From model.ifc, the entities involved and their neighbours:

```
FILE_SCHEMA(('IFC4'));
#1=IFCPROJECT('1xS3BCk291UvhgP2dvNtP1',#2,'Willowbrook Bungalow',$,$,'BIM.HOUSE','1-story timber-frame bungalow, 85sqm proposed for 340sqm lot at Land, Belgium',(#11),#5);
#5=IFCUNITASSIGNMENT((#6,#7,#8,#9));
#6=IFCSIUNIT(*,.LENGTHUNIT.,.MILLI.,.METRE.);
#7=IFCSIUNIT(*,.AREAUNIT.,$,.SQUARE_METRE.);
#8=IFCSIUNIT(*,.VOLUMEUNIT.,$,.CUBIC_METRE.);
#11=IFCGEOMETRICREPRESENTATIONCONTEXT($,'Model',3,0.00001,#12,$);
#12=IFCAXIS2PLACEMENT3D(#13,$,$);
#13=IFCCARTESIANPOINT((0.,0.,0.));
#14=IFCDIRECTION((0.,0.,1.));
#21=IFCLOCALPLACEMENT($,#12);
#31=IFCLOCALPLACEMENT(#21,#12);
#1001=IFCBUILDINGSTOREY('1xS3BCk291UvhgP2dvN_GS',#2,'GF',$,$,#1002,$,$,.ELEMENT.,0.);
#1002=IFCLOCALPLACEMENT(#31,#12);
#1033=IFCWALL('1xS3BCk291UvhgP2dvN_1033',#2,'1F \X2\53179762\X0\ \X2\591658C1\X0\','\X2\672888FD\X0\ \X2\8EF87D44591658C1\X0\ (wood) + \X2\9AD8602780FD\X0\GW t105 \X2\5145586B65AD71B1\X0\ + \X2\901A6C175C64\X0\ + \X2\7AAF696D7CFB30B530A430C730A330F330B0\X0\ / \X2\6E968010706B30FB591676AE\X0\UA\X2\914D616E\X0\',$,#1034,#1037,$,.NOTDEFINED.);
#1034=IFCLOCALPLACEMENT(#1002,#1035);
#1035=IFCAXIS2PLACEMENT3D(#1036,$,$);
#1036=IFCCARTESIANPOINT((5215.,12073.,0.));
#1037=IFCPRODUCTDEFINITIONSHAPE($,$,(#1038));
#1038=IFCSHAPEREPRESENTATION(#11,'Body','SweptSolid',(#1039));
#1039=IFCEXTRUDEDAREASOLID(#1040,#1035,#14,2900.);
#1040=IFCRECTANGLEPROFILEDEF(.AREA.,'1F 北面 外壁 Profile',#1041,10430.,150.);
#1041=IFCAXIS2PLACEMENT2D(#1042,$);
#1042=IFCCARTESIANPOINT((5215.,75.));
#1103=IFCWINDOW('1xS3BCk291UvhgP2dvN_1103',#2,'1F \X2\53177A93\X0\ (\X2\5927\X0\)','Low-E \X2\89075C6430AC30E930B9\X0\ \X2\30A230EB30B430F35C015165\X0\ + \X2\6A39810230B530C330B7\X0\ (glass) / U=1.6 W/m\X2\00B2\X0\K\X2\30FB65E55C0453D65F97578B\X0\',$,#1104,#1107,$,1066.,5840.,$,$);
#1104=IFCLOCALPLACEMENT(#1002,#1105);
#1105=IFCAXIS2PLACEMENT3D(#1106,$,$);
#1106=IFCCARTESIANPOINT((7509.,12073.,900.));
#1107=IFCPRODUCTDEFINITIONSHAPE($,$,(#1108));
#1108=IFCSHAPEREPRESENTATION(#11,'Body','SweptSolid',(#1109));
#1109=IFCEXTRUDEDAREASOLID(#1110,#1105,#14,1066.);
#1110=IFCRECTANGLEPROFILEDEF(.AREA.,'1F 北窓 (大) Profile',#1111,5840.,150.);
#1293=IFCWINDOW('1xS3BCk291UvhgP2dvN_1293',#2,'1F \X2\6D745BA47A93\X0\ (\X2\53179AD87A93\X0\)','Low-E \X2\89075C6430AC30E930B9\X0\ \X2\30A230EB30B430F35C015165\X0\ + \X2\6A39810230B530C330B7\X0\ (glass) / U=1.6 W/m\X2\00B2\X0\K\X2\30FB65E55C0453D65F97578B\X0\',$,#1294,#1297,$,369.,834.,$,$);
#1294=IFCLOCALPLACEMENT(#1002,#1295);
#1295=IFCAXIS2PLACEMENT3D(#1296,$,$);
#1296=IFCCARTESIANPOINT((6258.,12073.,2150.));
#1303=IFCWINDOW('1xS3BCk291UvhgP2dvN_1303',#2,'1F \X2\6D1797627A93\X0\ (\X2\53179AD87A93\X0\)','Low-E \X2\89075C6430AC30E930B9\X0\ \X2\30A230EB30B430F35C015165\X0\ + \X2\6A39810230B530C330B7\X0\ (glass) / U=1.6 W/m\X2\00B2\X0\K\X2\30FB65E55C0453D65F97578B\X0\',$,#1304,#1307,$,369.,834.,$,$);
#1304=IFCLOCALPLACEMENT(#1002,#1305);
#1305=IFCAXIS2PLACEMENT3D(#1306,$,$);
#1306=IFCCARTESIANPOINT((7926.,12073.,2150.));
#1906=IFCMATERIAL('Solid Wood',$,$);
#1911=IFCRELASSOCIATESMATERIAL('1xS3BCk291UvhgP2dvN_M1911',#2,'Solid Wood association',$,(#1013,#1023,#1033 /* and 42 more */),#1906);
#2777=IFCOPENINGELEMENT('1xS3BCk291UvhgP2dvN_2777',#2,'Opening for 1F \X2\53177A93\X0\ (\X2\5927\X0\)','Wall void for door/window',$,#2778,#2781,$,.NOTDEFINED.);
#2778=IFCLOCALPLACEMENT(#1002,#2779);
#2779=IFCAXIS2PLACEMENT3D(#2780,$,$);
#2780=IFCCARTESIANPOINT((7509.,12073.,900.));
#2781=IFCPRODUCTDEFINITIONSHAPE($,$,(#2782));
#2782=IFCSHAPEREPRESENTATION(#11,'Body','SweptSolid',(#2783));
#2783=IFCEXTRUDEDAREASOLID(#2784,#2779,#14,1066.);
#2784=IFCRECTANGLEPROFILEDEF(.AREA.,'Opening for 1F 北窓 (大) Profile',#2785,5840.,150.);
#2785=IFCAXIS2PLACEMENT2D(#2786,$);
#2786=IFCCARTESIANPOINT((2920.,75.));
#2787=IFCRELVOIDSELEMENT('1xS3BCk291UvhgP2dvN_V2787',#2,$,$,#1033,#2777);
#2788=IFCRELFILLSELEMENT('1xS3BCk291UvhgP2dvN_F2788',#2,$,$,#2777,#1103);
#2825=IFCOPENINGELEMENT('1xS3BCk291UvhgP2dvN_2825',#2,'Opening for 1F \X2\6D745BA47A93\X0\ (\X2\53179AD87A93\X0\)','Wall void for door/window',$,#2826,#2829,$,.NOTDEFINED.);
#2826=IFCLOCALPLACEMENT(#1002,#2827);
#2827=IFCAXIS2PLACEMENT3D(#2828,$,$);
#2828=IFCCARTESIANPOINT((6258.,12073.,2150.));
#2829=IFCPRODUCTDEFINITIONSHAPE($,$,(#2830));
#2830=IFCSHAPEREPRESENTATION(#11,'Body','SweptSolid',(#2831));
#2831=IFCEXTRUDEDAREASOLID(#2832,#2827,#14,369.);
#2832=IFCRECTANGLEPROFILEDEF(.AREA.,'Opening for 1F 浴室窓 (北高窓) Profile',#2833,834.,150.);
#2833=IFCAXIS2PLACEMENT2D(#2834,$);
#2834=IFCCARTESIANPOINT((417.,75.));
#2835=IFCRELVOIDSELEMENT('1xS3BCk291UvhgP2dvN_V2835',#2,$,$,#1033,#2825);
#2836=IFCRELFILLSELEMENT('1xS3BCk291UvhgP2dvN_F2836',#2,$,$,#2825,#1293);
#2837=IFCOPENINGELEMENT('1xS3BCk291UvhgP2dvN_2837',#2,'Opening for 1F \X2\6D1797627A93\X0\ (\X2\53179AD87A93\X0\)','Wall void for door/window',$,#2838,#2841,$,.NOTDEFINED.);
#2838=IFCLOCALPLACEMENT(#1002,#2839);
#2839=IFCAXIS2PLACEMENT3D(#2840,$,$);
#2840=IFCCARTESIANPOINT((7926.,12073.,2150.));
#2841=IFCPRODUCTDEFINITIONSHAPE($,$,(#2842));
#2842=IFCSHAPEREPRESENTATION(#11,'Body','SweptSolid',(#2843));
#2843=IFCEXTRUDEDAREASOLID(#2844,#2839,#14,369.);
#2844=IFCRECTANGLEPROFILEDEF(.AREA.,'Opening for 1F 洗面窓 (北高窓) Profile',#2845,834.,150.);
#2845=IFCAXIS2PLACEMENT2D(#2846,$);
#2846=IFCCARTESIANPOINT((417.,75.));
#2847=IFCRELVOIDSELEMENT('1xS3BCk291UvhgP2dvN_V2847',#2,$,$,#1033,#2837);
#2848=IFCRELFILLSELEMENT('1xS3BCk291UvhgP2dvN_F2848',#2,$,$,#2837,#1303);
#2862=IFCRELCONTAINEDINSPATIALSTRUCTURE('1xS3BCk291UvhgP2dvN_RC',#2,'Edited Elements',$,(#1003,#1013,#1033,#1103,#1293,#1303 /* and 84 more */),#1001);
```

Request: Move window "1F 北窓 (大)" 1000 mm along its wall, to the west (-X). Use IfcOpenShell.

```python
import ifcopenshell
import ifcopenshell.api.geometry
import ifcopenshell.util.placement
import ifcopenshell.util.unit

model = ifcopenshell.open("model.ifc")
unit_scale = ifcopenshell.util.unit.calculate_unit_scale(model)

window = model.by_id(1103)
opening = window.FillsVoids[0].RelatingOpeningElement
wall = opening.VoidsElements[0].RelatingBuildingElement

wall_matrix = ifcopenshell.util.placement.get_local_placement(wall.ObjectPlacement)
shift = wall_matrix[:3, 0] * -1 / unit_scale
before = ifcopenshell.util.placement.get_local_placement(window.ObjectPlacement)[:3, 3].copy()

# The window is not placed relative to its opening, so move both.
for product in (opening, window):
    matrix = ifcopenshell.util.placement.get_local_placement(product.ObjectPlacement)
    matrix[:3, 3] += shift
    ifcopenshell.api.geometry.edit_object_placement(model, product=product, matrix=matrix, is_si=False)

after = ifcopenshell.util.placement.get_local_placement(window.ObjectPlacement)[:3, 3]
print("window moved by", (after - before).round(3) + 0.0)

model.write("model_v2.ifc")
```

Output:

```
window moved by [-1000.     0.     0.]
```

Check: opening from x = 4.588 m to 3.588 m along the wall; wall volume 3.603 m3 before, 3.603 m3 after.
